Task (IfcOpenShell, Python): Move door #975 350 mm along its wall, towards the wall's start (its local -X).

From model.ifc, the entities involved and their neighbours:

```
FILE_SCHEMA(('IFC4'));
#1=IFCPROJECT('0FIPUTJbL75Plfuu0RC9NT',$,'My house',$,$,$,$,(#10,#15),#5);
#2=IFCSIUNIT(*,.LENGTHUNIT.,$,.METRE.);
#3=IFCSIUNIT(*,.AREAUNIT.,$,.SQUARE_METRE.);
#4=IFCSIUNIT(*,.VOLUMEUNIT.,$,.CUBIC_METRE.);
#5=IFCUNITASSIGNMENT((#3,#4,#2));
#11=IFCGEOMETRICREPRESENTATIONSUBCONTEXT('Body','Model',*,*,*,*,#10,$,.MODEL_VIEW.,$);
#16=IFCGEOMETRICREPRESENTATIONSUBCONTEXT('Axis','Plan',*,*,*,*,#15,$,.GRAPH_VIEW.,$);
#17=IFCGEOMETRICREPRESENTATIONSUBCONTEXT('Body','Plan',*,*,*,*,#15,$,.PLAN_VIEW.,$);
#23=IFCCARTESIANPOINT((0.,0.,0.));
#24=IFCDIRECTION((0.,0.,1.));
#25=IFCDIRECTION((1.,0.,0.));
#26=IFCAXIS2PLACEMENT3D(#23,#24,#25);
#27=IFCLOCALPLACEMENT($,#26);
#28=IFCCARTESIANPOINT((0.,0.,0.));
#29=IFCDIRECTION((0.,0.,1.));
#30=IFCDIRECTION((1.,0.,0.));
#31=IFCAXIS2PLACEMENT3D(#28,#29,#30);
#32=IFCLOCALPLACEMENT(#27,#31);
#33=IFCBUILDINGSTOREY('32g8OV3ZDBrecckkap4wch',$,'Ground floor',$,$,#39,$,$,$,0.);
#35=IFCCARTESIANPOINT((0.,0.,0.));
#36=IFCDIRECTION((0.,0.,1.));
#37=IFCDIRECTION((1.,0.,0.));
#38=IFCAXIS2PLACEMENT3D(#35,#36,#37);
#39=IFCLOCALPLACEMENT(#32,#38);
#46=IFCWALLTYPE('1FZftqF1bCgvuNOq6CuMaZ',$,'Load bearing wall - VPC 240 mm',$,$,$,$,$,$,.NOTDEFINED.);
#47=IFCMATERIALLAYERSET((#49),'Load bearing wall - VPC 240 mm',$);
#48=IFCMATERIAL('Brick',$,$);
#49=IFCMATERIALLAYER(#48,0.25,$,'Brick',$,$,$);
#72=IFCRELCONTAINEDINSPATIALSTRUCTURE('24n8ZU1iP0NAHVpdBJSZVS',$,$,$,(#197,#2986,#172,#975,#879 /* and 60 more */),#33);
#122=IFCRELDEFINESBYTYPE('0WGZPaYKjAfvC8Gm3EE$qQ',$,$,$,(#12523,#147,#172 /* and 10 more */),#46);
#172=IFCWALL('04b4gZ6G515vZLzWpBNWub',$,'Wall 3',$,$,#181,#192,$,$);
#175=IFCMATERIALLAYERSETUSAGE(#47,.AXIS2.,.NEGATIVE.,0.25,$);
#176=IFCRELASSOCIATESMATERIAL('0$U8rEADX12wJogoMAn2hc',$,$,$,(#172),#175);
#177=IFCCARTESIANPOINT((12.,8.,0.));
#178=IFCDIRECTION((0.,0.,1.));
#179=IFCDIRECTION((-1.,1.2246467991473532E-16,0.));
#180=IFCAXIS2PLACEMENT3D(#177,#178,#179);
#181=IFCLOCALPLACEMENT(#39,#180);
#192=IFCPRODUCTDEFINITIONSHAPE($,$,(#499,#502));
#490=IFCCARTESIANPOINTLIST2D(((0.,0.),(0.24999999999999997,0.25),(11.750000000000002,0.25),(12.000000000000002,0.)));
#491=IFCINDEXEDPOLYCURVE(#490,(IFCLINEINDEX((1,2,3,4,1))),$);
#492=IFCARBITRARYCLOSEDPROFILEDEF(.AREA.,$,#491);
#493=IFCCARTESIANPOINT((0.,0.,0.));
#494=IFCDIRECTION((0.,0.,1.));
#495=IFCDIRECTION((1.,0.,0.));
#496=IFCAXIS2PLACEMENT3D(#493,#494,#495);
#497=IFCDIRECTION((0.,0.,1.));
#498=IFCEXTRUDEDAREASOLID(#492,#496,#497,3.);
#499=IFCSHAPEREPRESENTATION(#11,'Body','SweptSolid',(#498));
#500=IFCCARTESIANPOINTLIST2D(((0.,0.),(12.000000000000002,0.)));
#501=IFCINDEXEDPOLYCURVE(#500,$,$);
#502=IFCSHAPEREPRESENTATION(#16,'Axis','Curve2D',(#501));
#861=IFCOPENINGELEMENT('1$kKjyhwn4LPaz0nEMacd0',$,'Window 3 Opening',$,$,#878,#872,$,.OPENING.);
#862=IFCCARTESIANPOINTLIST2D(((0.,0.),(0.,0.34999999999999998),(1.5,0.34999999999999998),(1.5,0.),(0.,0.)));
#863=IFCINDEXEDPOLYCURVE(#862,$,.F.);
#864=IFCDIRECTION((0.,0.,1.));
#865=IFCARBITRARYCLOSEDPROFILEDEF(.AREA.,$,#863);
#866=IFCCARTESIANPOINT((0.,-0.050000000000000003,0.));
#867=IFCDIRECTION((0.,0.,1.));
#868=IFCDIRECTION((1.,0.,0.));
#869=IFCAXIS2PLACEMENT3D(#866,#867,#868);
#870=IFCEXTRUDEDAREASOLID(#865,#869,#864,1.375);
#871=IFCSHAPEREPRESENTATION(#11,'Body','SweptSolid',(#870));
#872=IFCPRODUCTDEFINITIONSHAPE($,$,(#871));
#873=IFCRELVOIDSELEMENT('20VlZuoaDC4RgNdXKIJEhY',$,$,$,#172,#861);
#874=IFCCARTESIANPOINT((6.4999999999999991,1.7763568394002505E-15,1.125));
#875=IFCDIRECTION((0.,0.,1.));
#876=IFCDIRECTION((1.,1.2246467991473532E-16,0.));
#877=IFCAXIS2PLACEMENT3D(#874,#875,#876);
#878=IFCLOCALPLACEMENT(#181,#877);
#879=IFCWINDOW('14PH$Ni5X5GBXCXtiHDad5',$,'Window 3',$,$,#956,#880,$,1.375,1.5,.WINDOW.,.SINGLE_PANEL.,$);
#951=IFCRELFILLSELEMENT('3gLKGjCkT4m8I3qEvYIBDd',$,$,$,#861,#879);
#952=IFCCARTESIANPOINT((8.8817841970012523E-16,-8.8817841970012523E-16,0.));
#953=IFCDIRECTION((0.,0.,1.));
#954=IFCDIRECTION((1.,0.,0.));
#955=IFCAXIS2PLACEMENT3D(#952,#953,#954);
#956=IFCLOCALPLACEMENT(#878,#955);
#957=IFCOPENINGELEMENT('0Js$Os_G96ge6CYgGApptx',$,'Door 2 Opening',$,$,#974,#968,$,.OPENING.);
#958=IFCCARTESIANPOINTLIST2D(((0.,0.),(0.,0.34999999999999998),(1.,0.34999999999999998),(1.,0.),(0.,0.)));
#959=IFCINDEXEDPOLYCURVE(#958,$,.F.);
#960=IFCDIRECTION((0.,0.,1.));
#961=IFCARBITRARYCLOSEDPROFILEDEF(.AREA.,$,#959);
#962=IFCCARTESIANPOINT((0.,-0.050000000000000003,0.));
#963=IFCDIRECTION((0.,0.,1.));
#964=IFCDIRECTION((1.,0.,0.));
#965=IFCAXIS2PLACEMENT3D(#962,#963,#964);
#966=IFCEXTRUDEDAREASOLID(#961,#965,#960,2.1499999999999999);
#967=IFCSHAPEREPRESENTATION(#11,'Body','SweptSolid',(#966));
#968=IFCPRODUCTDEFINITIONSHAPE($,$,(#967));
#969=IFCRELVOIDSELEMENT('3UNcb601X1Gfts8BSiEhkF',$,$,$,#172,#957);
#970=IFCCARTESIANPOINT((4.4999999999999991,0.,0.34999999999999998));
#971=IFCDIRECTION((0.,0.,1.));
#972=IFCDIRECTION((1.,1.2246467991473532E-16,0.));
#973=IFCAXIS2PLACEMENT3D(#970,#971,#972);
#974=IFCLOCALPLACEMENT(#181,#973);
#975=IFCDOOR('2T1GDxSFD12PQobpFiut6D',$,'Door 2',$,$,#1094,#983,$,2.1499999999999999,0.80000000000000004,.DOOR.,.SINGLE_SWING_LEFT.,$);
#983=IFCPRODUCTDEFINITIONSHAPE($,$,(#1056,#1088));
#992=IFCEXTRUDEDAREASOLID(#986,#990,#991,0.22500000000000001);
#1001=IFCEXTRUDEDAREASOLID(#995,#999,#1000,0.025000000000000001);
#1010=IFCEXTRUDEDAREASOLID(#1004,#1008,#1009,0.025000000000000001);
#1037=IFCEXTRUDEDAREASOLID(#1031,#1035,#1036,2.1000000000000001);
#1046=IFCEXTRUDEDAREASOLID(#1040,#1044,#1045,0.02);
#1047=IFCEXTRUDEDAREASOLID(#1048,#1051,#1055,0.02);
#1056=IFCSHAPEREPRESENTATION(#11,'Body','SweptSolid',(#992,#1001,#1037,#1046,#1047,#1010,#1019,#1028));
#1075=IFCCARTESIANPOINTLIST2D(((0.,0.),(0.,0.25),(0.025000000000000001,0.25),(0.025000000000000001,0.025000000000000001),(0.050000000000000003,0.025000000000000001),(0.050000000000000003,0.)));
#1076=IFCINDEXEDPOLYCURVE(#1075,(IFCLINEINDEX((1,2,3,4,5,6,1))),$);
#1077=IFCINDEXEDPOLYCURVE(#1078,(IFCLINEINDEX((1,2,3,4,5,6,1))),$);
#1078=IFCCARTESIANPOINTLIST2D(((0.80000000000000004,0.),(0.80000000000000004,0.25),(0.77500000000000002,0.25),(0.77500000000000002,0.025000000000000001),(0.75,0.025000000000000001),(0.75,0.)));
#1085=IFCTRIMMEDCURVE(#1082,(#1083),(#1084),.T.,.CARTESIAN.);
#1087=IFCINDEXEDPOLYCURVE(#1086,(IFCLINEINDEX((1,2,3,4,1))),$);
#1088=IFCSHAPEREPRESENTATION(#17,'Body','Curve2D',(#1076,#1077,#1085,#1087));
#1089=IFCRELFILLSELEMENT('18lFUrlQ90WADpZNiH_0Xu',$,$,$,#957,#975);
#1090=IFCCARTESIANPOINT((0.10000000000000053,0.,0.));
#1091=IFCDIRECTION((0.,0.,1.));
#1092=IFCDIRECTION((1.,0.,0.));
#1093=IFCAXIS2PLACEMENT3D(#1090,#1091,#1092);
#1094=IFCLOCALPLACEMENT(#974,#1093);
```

```python
import ifcopenshell
import ifcopenshell.api.geometry
import ifcopenshell.util.placement

model = ifcopenshell.open("model.ifc")

door = model.by_guid("2T1GDxSFD12PQobpFiut6D")
opening = door.FillsVoids[0].RelatingOpeningElement
wall = opening.VoidsElements[0].RelatingBuildingElement

wall_matrix = ifcopenshell.util.placement.get_local_placement(wall.ObjectPlacement)
shift = wall_matrix[:3, 0] * -0.35
before = ifcopenshell.util.placement.get_local_placement(door.ObjectPlacement)[:3, 3].copy()

# The door is placed relative to its opening, so it follows when the opening moves.
matrix = ifcopenshell.util.placement.get_local_placement(opening.ObjectPlacement)
matrix[:3, 3] += shift
ifcopenshell.api.geometry.edit_object_placement(
    model, product=opening, matrix=matrix, is_si=False, should_transform_children=True
)

after = ifcopenshell.util.placement.get_local_placement(door.ObjectPlacement)[:3, 3]
print("door moved by", (after - before).round(3) + 0.0)

model.write("model_updated.ifc")
```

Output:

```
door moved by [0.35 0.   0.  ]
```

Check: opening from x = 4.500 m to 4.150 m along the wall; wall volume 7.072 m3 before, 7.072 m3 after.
